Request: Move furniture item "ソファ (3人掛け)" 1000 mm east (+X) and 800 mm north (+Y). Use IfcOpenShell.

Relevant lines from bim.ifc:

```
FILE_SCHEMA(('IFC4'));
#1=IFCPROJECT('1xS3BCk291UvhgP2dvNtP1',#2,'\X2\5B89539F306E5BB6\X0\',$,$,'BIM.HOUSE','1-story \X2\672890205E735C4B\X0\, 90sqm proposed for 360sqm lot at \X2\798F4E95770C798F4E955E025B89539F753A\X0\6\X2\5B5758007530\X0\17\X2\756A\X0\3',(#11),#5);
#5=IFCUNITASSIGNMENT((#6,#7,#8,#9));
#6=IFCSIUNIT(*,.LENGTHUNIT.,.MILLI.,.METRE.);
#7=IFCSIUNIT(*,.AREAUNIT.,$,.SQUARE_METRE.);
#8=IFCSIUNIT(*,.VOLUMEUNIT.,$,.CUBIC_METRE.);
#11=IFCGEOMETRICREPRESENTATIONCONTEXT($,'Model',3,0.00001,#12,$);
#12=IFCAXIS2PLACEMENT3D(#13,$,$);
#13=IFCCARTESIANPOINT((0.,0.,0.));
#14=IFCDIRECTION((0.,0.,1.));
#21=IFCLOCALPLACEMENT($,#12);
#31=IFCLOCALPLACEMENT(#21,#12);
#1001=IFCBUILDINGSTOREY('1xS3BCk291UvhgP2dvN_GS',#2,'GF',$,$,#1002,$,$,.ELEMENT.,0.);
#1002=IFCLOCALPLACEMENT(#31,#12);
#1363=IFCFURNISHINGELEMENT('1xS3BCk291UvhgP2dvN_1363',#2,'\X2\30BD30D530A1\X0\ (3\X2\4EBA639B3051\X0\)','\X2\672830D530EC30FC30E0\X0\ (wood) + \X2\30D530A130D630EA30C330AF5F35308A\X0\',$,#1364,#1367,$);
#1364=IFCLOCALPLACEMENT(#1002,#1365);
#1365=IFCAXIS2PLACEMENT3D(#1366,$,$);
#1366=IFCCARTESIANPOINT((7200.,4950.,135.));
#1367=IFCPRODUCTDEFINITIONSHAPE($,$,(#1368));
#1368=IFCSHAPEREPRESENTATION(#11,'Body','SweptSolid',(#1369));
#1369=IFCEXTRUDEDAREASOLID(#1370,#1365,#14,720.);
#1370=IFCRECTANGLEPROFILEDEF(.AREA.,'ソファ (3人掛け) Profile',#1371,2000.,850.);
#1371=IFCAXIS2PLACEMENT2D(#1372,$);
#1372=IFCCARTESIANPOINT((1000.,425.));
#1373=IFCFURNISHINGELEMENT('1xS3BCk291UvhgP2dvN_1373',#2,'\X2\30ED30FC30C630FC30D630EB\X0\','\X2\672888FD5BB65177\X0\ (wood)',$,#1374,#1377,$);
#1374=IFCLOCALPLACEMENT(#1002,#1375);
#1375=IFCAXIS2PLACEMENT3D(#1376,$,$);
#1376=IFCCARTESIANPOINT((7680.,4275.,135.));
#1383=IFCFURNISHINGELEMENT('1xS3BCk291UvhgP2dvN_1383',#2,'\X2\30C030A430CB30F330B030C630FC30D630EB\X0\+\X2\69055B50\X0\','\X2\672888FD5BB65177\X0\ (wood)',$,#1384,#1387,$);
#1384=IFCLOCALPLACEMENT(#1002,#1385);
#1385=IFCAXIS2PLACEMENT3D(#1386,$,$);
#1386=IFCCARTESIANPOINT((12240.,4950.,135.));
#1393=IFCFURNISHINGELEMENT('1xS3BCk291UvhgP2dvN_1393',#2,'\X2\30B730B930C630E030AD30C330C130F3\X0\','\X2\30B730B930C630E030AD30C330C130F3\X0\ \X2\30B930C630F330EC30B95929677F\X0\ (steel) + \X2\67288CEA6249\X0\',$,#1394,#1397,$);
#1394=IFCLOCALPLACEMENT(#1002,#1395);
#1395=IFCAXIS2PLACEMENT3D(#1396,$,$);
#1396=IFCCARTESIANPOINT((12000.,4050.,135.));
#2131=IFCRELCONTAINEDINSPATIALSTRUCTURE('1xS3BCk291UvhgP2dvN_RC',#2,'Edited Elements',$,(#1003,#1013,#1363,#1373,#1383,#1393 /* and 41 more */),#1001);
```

```python
import ifcopenshell
import ifcopenshell.api.geometry
import ifcopenshell.util.placement

model = ifcopenshell.open("bim.ifc")

item = model.by_guid("1xS3BCk291UvhgP2dvN_1363")
matrix = ifcopenshell.util.placement.get_local_placement(item.ObjectPlacement)
matrix[0, 3] += 1000.0
matrix[1, 3] += 800.0
ifcopenshell.api.geometry.edit_object_placement(model, product=item, matrix=matrix, is_si=False)

print(ifcopenshell.util.placement.get_local_placement(item.ObjectPlacement).round(3) + 0.0)

model.write("bim_v2.ifc")
```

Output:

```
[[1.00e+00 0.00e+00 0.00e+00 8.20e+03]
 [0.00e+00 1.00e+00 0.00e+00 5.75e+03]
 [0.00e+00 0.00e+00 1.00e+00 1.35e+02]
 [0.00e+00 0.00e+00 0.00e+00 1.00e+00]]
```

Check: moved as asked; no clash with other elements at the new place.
